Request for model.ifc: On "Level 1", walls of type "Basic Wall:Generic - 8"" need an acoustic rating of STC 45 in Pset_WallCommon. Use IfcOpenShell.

First a look at what the model holds.

```python
import ifcopenshell
import ifcopenshell.util.element

model = ifcopenshell.open("model.ifc")
print(model.schema)
storey = next(s for s in model.by_type("IfcBuildingStorey") if s.Name == "Level 1")
walls = [e for e in ifcopenshell.util.element.get_decomposition(storey) if e.is_a("IfcWall")]
seen = {}
for e in walls:
    element_type = ifcopenshell.util.element.get_type(e)
    key = (element_type.Name if element_type != e and element_type else None, ifcopenshell.util.element.get_pset(e, "Pset_WallCommon", "AcousticRating"))
    seen[key] = seen.get(key, 0) + 1
for (name, value), count in sorted(seen.items(), key=str):
    print(count, "x", name, "|", value)
```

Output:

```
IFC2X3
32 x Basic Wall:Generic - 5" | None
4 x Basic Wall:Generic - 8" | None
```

```python
import ifcopenshell
import ifcopenshell.api.pset
import ifcopenshell.util.element

model = ifcopenshell.open("model.ifc")

storey = next(s for s in model.by_type("IfcBuildingStorey") if s.Name == "Level 1")
walls = [e for e in ifcopenshell.util.element.get_decomposition(storey) if e.is_a("IfcWall")]

count = 0
for e in walls:
    element_type = ifcopenshell.util.element.get_type(e)
    if element_type in (None, e) or element_type.Name != 'Basic Wall:Generic - 8"':
        continue
    # add_pset returns the element's existing set when there is one.
    pset = ifcopenshell.api.pset.add_pset(model, product=e, name="Pset_WallCommon")
    ifcopenshell.api.pset.edit_pset(model, pset=pset, properties={"AcousticRating": "STC 45"})
    count += 1

print(count, "walls updated")

model.write("model_edited.ifc")
```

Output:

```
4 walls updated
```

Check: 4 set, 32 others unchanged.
